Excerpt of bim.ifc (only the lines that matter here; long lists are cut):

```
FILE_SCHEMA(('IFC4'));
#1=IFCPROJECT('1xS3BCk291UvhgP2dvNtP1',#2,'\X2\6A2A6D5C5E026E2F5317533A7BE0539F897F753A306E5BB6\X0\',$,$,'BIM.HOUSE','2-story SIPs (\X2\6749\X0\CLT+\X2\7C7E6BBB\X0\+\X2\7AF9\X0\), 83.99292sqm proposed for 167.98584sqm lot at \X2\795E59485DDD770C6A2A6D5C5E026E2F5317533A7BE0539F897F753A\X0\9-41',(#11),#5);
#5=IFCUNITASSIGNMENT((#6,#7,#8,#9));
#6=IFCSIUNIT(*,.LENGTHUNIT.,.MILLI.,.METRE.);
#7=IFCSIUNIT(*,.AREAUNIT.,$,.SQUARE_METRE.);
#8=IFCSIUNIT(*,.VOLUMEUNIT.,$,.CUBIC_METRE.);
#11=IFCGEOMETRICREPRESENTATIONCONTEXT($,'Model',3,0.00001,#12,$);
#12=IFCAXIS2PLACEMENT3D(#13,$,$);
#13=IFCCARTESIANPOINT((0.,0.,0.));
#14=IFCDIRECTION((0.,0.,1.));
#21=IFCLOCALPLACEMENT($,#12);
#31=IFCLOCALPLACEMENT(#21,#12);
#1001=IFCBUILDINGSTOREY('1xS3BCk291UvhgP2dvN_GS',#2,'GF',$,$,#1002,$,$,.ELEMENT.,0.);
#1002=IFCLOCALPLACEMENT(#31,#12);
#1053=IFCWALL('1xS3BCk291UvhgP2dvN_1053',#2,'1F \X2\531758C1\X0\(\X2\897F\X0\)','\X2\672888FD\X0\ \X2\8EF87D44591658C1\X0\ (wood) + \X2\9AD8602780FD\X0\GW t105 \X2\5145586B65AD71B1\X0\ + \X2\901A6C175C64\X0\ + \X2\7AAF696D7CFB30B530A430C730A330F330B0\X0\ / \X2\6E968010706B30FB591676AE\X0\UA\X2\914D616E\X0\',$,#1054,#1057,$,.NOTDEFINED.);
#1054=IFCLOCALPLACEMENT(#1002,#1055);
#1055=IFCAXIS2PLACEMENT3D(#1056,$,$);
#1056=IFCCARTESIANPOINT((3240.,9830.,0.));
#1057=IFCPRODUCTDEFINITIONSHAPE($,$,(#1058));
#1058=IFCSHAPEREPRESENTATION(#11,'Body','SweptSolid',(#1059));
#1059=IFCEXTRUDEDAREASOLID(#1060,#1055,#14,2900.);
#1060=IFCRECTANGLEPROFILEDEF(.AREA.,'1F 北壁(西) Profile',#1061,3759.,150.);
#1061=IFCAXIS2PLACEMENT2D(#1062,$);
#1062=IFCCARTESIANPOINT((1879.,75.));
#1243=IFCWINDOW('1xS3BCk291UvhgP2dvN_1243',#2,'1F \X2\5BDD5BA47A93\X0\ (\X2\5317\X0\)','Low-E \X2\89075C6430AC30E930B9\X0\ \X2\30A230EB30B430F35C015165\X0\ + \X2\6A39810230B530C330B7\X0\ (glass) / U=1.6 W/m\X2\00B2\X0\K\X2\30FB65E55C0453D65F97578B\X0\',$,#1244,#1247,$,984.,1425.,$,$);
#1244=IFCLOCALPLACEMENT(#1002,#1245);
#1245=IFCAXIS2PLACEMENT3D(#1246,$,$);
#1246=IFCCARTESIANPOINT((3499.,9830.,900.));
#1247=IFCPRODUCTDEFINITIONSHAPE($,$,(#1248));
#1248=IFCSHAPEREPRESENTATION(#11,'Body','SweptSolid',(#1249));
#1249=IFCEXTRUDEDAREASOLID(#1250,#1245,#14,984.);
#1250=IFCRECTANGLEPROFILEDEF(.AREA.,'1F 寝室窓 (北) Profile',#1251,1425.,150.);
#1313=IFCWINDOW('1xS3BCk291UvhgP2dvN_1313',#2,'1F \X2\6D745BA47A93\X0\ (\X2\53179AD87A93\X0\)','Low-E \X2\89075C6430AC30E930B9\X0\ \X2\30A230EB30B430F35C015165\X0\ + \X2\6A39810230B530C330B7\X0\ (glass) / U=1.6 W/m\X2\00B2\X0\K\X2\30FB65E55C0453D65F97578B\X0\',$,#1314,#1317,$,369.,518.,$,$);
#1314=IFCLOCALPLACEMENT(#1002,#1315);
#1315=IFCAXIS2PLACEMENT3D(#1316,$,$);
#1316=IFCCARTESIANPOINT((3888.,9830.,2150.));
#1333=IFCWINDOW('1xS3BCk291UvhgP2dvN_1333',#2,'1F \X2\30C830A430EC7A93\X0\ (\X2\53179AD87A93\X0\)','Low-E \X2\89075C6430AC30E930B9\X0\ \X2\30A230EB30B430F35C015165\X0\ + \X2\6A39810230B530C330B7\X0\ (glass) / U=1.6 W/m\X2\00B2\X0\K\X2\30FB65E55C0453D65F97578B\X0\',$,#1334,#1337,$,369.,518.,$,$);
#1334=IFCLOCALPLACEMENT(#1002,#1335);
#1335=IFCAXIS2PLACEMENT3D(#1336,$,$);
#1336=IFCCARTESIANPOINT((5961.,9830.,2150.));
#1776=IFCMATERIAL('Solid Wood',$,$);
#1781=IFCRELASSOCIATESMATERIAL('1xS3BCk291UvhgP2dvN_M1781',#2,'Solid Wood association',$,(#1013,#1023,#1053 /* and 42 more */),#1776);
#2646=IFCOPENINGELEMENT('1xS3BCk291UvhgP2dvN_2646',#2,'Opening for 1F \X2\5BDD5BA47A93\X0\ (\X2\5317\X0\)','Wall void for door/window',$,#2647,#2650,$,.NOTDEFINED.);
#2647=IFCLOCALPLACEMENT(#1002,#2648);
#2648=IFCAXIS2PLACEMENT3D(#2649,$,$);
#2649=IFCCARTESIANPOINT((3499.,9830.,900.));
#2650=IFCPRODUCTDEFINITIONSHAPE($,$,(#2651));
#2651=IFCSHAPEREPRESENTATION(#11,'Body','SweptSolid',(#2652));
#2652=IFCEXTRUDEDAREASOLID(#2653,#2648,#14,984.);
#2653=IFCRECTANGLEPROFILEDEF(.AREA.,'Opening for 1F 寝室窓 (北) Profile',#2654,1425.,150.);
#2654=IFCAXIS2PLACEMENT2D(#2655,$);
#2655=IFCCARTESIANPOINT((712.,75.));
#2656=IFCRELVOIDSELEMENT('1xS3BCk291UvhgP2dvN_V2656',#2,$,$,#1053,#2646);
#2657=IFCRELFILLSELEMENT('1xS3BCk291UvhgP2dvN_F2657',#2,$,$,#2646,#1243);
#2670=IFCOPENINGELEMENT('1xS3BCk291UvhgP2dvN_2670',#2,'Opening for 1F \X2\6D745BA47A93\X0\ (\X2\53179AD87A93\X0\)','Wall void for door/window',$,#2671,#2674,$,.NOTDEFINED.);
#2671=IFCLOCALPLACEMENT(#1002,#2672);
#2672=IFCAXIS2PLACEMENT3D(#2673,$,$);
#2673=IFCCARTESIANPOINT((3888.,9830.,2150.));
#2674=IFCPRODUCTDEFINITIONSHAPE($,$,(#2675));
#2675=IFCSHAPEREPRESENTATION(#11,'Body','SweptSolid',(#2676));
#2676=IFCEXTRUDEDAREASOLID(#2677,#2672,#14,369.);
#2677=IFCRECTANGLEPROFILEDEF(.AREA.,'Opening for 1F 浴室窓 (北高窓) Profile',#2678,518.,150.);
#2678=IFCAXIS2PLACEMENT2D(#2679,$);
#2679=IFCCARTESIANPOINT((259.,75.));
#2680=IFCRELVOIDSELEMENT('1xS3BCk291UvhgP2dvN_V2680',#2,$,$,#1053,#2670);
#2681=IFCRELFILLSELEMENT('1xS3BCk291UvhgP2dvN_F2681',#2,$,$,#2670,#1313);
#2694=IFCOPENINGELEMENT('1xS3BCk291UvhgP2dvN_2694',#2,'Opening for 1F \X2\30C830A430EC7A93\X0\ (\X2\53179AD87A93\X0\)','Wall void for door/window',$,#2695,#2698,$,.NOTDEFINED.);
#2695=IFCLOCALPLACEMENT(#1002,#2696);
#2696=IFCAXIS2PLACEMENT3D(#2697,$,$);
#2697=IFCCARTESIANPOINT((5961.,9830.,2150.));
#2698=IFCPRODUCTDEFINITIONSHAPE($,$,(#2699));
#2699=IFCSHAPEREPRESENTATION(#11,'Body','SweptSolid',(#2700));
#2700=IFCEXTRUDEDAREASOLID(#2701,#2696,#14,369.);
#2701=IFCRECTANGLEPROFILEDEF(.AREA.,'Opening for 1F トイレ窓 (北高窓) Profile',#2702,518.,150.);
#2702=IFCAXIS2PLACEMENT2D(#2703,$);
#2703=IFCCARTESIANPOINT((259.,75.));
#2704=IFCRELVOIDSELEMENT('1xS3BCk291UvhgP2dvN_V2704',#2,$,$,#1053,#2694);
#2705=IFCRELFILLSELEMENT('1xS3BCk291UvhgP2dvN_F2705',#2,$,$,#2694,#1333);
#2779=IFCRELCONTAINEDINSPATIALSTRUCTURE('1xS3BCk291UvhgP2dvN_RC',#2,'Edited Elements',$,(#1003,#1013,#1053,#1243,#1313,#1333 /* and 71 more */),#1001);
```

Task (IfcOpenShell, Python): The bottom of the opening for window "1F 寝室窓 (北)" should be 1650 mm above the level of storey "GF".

```python
import numpy as np
import ifcopenshell
import ifcopenshell.api.geometry
import ifcopenshell.geom
import ifcopenshell.util.element
import ifcopenshell.util.placement
import ifcopenshell.util.shape
import ifcopenshell.util.unit

model = ifcopenshell.open("bim.ifc")
unit_scale = ifcopenshell.util.unit.calculate_unit_scale(model)

window = model.by_guid("1xS3BCk291UvhgP2dvN_1243")
opening = window.FillsVoids[0].RelatingOpeningElement
storey = ifcopenshell.util.element.get_container(window, ifc_class="IfcBuildingStorey")
level = ifcopenshell.util.placement.get_local_placement(storey.ObjectPlacement)[2, 3]

# The opening's origin need not be at the sill, so measure its lowest point.
shape = ifcopenshell.geom.create_shape(ifcopenshell.geom.settings(), opening)
bottom = ifcopenshell.util.shape.get_shape_bottom_elevation(shape, shape.geometry) / unit_scale
dz = level + 1650.0 - bottom

shift = np.array([0.0, 0.0, dz])
# The window is not placed relative to its opening, so move both.
for product in (opening, window):
    matrix = ifcopenshell.util.placement.get_local_placement(product.ObjectPlacement)
    matrix[:3, 3] += shift
    ifcopenshell.api.geometry.edit_object_placement(model, product=product, matrix=matrix, is_si=False)

print(f"moved by {dz * unit_scale:+.3f} m")

model.write("bim-out.ifc")
```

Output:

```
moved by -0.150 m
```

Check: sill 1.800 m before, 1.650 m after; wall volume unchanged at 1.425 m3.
